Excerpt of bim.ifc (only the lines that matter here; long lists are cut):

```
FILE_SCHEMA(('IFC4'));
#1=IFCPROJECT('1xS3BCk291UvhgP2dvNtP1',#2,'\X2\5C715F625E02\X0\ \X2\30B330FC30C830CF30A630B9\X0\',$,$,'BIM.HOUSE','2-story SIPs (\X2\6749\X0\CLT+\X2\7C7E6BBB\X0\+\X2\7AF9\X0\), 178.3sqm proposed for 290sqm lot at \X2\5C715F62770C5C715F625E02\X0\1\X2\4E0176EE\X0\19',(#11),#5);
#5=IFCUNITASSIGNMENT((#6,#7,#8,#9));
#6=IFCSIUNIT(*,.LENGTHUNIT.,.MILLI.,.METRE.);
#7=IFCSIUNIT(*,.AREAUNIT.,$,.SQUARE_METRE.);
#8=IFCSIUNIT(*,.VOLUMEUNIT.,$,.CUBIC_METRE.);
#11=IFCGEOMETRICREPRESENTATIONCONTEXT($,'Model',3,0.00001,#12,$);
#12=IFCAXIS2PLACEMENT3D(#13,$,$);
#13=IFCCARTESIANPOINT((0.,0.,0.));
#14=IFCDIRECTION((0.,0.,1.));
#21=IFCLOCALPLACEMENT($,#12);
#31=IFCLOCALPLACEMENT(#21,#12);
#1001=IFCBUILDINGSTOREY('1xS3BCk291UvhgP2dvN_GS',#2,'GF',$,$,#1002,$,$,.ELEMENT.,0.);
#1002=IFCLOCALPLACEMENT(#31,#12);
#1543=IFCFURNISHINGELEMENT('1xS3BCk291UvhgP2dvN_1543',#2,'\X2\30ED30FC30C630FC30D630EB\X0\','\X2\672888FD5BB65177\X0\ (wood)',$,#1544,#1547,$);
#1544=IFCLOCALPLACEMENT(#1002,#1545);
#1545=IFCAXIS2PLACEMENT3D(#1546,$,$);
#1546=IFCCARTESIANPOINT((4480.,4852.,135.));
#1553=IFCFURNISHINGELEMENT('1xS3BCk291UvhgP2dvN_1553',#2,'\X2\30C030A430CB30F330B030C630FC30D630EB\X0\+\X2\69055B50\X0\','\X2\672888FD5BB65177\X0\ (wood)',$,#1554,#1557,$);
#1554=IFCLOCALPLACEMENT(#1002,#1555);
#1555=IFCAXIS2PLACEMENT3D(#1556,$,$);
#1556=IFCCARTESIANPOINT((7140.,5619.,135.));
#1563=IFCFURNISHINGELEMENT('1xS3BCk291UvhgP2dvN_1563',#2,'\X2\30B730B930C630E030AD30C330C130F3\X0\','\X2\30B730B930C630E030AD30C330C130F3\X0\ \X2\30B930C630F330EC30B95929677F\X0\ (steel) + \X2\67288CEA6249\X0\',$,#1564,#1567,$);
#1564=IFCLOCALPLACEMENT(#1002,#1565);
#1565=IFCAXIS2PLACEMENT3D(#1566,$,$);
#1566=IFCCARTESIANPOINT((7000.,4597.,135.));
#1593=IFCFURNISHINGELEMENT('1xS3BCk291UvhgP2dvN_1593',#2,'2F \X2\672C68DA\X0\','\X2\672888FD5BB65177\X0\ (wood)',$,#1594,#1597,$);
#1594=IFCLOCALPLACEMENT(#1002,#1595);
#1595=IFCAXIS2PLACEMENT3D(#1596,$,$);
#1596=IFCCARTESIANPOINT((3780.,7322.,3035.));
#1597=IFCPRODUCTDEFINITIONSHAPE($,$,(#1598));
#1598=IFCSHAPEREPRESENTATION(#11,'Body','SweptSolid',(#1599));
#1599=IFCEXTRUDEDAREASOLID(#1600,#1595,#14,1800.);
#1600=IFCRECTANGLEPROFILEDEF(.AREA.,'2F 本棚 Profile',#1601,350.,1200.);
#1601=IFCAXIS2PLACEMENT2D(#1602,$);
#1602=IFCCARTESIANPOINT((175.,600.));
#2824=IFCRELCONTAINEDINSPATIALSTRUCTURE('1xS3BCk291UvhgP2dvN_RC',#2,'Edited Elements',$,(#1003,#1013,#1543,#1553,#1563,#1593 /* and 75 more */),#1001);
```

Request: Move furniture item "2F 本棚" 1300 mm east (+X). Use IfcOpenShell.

```python
import ifcopenshell
import ifcopenshell.api.geometry
import ifcopenshell.util.placement
import ifcopenshell.util.unit

model = ifcopenshell.open("bim.ifc")
unit_scale = ifcopenshell.util.unit.calculate_unit_scale(model)

item = model.by_guid("1xS3BCk291UvhgP2dvN_1593")
matrix = ifcopenshell.util.placement.get_local_placement(item.ObjectPlacement)
matrix[0, 3] += 1.3 / unit_scale
ifcopenshell.api.geometry.edit_object_placement(model, product=item, matrix=matrix, is_si=False)

print(ifcopenshell.util.placement.get_local_placement(item.ObjectPlacement).round(3) + 0.0)

model.write("bim_edited.ifc")
```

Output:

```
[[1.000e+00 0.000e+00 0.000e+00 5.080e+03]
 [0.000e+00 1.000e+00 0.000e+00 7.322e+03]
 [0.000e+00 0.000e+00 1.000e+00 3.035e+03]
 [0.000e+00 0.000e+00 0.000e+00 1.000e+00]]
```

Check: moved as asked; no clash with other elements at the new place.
